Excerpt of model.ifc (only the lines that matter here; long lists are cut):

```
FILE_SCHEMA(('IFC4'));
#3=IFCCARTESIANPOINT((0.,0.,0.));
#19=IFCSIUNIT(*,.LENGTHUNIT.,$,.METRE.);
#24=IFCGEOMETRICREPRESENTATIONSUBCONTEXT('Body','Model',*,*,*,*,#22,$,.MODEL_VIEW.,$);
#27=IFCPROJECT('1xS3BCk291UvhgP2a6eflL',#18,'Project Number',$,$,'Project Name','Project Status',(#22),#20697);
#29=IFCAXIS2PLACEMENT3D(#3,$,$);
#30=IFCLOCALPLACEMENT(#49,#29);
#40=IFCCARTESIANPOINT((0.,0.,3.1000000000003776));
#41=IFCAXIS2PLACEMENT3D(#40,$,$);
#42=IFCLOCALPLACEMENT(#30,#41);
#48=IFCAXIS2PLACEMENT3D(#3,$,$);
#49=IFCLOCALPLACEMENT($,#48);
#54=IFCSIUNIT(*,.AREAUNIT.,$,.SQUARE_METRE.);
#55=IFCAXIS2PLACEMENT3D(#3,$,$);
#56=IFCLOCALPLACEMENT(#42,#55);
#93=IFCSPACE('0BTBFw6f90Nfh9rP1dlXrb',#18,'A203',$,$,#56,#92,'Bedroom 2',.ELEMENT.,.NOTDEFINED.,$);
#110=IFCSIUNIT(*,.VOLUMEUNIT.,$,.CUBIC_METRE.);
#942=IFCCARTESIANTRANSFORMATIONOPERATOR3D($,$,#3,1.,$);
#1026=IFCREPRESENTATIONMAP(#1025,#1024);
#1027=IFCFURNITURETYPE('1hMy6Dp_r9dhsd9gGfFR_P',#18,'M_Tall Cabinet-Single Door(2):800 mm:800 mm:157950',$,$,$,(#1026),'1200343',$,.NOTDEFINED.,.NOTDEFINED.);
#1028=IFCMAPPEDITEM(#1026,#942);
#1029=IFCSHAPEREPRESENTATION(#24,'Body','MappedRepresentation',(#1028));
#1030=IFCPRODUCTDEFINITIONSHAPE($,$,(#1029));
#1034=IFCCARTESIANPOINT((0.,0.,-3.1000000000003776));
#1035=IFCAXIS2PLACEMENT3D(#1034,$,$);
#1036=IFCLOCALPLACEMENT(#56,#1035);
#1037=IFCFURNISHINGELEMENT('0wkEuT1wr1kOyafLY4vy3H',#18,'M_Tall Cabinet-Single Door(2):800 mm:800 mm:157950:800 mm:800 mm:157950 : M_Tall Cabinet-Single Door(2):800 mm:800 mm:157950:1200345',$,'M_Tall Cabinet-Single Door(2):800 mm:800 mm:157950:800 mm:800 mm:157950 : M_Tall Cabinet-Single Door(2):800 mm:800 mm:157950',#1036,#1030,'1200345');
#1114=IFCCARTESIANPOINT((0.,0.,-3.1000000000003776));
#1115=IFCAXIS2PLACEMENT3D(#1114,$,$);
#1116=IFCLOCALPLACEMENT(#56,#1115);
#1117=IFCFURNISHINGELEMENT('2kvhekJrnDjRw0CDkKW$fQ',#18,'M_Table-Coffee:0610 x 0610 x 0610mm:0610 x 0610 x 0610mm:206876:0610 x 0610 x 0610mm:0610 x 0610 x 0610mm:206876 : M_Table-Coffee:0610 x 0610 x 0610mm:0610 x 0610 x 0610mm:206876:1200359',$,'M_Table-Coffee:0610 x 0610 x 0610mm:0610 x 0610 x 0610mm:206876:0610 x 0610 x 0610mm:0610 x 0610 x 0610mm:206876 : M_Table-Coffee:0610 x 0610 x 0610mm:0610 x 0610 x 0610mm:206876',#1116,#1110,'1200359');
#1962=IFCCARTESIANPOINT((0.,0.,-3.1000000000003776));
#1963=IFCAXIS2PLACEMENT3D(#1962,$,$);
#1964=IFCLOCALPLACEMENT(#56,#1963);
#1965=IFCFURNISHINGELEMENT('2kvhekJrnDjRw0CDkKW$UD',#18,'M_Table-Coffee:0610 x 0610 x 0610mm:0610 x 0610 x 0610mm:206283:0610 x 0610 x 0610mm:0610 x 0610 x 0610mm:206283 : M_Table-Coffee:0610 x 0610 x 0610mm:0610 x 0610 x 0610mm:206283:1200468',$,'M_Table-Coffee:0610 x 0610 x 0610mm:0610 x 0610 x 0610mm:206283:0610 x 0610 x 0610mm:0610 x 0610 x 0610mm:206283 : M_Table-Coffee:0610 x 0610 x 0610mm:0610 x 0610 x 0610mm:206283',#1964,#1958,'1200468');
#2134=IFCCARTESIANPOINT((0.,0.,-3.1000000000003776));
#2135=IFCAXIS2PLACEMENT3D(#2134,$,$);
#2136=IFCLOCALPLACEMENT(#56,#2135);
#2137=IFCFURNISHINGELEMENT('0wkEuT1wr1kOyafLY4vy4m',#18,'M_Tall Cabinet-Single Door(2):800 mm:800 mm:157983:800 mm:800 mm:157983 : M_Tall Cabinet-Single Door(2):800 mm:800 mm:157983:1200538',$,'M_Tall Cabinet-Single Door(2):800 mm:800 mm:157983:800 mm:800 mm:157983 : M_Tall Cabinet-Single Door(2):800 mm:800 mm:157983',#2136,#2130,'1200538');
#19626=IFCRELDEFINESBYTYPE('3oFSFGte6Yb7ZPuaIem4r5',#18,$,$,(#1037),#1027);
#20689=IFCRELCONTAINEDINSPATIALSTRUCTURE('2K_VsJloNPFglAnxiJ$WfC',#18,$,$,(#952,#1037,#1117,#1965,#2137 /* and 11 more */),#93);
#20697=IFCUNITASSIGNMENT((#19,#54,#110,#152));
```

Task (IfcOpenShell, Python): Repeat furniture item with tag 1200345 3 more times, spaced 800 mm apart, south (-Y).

```python
import numpy as np
import ifcopenshell
import ifcopenshell.api.geometry
import ifcopenshell.api.root
import ifcopenshell.util.element
import ifcopenshell.util.placement

model = ifcopenshell.open("model.ifc")


def reuse_history(source, copy):
    """copy_class also copies each property set's owner history, people and application; keep the originals."""
    for rel in copy.IsDefinedBy:
        if rel.is_a("IfcRelDefinesByProperties") and (history := rel.RelatingPropertyDefinition.OwnerHistory):
            rel.RelatingPropertyDefinition.OwnerHistory = source.OwnerHistory
            ifcopenshell.util.element.remove_deep2(model, history)


source = model.by_id(1037)
base = ifcopenshell.util.placement.get_local_placement(source.ObjectPlacement)
step = np.array([0.0, -1.0, 0.0]) * 0.8

for i in range(1, 4):
    copy = ifcopenshell.api.root.copy_class(model, product=source)
    copy.Representation = ifcopenshell.util.element.copy_deep(
        model, source.Representation, exclude=["IfcGeometricRepresentationContext", "IfcRepresentationMap"]
    )
    copy.Name = "M_Tall Cabinet-Single Door(2):800 mm:800 mm:157950:800 mm:800 mm:157950 : M_Tall Cabinet-Single Door(2):800 mm:800 mm"
    copy.Tag = None
    reuse_history(source, copy)
    matrix = base.copy()
    matrix[:3, 3] += i * step
    print("added at", matrix[:3, 3].round(3) + 0.0)
    ifcopenshell.api.geometry.edit_object_placement(model, product=copy, matrix=matrix, is_si=False)

model.write("model_edited.ifc")
```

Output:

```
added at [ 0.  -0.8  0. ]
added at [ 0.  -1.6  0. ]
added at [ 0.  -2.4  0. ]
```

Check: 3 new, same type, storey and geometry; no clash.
